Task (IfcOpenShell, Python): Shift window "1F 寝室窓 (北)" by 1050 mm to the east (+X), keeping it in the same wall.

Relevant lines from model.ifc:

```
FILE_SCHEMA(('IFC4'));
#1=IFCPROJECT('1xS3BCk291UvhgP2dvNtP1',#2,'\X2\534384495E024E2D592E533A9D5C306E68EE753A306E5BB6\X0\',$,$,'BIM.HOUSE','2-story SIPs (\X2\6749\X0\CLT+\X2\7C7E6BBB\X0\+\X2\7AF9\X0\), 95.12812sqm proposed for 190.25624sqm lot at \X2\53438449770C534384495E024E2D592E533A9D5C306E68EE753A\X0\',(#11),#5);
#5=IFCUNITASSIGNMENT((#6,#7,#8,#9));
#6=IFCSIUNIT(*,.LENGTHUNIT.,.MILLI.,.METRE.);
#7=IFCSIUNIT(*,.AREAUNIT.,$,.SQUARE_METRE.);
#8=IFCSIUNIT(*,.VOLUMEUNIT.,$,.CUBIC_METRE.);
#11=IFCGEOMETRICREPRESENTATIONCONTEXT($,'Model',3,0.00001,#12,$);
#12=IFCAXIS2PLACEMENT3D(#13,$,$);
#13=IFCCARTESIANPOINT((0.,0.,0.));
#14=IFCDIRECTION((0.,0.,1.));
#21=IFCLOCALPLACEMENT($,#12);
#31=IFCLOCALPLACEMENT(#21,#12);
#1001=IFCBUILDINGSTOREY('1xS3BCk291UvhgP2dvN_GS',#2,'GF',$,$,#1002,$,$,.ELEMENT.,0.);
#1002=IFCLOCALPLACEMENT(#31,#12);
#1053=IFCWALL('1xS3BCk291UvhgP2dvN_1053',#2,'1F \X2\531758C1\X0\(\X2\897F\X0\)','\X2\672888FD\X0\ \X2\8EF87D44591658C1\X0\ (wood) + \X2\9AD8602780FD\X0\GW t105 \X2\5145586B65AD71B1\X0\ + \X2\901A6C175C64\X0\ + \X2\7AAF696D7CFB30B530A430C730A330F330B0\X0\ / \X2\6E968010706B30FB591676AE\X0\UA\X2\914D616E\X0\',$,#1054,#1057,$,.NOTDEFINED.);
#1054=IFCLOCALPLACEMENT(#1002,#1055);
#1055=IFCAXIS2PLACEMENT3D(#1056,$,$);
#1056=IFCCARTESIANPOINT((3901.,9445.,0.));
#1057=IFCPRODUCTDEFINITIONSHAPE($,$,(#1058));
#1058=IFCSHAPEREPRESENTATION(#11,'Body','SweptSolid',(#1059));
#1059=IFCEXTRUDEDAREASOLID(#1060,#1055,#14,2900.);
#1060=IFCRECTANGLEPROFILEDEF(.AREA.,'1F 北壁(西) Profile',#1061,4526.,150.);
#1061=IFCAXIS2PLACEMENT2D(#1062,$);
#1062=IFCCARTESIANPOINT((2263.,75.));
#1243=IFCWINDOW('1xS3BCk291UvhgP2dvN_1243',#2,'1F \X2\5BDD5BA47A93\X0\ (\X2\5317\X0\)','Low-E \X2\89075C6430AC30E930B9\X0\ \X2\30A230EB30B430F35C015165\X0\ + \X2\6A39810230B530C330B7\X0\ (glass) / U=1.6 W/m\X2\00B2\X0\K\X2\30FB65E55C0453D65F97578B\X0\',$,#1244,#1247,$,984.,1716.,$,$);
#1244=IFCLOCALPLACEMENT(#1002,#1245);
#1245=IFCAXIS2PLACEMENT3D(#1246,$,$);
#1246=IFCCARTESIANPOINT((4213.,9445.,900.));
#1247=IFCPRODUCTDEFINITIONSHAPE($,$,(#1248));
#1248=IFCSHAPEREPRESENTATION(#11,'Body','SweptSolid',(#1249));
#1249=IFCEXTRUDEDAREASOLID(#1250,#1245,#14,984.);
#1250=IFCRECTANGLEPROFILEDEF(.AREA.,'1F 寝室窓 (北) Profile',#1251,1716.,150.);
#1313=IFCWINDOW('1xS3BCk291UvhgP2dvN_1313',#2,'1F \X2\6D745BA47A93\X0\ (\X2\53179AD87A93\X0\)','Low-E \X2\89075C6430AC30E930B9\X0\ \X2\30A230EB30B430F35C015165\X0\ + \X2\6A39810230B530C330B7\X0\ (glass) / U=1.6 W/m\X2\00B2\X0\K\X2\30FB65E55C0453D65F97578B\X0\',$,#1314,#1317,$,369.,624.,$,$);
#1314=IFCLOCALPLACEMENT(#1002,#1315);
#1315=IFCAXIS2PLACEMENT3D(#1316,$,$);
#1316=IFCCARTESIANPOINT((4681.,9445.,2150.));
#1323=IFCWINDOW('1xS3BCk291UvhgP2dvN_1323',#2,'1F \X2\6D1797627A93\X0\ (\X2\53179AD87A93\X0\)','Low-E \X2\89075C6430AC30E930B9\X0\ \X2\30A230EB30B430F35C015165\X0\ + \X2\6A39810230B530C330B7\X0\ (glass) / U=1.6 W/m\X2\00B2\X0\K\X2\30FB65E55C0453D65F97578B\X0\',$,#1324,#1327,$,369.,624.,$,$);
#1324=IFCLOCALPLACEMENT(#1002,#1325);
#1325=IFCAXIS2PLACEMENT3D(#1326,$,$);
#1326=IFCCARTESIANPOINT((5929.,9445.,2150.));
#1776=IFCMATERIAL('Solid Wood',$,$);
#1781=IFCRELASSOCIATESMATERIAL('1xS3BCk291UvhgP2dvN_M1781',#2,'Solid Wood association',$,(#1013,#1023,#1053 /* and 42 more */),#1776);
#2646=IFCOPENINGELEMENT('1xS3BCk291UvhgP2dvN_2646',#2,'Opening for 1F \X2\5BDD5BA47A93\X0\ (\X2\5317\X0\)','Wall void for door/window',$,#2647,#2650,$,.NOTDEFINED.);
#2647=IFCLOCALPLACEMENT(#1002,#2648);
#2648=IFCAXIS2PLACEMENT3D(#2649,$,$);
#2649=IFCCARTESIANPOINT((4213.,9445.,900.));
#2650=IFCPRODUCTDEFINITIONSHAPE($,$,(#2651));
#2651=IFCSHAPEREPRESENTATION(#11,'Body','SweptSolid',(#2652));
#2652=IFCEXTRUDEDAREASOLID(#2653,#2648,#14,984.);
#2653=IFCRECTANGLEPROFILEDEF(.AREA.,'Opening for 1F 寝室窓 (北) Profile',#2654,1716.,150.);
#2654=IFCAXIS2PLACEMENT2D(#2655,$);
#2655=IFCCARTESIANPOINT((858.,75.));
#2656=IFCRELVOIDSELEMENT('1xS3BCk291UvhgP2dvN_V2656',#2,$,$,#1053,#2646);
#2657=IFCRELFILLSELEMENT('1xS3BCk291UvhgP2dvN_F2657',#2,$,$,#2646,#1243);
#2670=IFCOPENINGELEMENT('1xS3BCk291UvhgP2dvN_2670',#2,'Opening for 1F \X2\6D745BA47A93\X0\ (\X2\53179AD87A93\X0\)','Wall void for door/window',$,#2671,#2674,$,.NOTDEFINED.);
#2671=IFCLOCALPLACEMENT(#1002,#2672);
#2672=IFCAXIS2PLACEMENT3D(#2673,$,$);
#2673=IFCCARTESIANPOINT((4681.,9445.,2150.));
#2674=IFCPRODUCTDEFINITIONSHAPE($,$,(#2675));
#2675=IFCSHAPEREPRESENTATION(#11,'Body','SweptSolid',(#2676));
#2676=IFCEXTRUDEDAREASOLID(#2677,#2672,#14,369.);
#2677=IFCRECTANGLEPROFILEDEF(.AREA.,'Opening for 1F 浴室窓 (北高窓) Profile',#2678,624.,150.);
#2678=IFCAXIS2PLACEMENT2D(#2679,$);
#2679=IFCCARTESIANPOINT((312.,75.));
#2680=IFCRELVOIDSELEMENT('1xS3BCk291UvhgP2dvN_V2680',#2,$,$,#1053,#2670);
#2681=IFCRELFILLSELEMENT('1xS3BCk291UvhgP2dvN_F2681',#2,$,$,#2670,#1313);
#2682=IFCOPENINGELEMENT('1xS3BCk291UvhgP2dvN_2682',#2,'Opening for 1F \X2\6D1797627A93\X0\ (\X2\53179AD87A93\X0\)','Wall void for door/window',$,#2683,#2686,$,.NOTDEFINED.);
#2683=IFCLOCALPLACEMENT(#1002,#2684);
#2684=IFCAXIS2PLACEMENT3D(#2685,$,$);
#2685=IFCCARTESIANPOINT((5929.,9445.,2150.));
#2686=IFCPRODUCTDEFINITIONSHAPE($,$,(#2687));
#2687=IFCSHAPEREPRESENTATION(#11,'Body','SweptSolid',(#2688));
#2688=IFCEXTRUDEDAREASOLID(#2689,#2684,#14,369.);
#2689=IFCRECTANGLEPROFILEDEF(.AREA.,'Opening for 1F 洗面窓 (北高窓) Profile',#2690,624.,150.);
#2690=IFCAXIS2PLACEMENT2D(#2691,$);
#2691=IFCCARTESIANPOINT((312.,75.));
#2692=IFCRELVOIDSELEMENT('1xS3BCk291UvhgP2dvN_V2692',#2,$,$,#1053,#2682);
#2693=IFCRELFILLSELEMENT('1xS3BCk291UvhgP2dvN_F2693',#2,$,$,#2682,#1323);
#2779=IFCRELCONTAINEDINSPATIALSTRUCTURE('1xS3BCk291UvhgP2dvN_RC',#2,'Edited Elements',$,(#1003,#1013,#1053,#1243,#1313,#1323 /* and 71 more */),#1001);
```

```python
import ifcopenshell
import ifcopenshell.api.geometry
import ifcopenshell.util.placement
import ifcopenshell.util.unit

model = ifcopenshell.open("model.ifc")
unit_scale = ifcopenshell.util.unit.calculate_unit_scale(model)

window = model.by_guid("1xS3BCk291UvhgP2dvN_1243")
opening = window.FillsVoids[0].RelatingOpeningElement
wall = opening.VoidsElements[0].RelatingBuildingElement

wall_matrix = ifcopenshell.util.placement.get_local_placement(wall.ObjectPlacement)
shift = wall_matrix[:3, 0] * 1.05 / unit_scale
before = ifcopenshell.util.placement.get_local_placement(window.ObjectPlacement)[:3, 3].copy()

# The window is not placed relative to its opening, so move both.
for product in (opening, window):
    matrix = ifcopenshell.util.placement.get_local_placement(product.ObjectPlacement)
    matrix[:3, 3] += shift
    ifcopenshell.api.geometry.edit_object_placement(model, product=product, matrix=matrix, is_si=False)

after = ifcopenshell.util.placement.get_local_placement(window.ObjectPlacement)[:3, 3]
print("window moved by", (after - before).round(3) + 0.0)

model.write("model_rev.ifc")
```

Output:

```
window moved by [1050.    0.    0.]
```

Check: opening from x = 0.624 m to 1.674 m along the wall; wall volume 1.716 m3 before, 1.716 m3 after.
